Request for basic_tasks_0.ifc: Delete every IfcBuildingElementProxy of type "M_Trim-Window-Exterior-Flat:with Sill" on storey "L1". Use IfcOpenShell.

First a look at what the model holds.

```python
import ifcopenshell
import ifcopenshell.util.element

model = ifcopenshell.open("basic_tasks_0.ifc")
print(model.schema)
storey = next(s for s in model.by_type("IfcBuildingStorey") if s.Name == "L1")
proxies = [e for e in ifcopenshell.util.element.get_decomposition(storey) if e.is_a("IfcBuildingElementProxy")]
seen = {}
for e in proxies:
    element_type = ifcopenshell.util.element.get_type(e)
    name = element_type.Name if element_type not in (None, e) else None
    seen[name] = seen.get(name, 0) + 1
for name, count in sorted(seen.items(), key=str):
    print(count, "x", name)
```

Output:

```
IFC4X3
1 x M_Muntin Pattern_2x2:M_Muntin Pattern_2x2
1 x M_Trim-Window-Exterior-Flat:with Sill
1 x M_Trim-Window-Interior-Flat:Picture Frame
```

```python
import ifcopenshell
import ifcopenshell.api.root
import ifcopenshell.util.element

model = ifcopenshell.open("basic_tasks_0.ifc")

storey = next(s for s in model.by_type("IfcBuildingStorey") if s.Name == "L1")
proxies = [e for e in ifcopenshell.util.element.get_decomposition(storey) if e.is_a("IfcBuildingElementProxy")]
targets = [e for e in proxies if (t := ifcopenshell.util.element.get_type(e)) not in (None, e) and t.Name == "M_Trim-Window-Exterior-Flat:with Sill"]

for e in targets:
    ifcopenshell.api.root.remove_product(model, product=e)
print(len(targets), "removed")

model.write("basic_tasks_0-out.ifc")
```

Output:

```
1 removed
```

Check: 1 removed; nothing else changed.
